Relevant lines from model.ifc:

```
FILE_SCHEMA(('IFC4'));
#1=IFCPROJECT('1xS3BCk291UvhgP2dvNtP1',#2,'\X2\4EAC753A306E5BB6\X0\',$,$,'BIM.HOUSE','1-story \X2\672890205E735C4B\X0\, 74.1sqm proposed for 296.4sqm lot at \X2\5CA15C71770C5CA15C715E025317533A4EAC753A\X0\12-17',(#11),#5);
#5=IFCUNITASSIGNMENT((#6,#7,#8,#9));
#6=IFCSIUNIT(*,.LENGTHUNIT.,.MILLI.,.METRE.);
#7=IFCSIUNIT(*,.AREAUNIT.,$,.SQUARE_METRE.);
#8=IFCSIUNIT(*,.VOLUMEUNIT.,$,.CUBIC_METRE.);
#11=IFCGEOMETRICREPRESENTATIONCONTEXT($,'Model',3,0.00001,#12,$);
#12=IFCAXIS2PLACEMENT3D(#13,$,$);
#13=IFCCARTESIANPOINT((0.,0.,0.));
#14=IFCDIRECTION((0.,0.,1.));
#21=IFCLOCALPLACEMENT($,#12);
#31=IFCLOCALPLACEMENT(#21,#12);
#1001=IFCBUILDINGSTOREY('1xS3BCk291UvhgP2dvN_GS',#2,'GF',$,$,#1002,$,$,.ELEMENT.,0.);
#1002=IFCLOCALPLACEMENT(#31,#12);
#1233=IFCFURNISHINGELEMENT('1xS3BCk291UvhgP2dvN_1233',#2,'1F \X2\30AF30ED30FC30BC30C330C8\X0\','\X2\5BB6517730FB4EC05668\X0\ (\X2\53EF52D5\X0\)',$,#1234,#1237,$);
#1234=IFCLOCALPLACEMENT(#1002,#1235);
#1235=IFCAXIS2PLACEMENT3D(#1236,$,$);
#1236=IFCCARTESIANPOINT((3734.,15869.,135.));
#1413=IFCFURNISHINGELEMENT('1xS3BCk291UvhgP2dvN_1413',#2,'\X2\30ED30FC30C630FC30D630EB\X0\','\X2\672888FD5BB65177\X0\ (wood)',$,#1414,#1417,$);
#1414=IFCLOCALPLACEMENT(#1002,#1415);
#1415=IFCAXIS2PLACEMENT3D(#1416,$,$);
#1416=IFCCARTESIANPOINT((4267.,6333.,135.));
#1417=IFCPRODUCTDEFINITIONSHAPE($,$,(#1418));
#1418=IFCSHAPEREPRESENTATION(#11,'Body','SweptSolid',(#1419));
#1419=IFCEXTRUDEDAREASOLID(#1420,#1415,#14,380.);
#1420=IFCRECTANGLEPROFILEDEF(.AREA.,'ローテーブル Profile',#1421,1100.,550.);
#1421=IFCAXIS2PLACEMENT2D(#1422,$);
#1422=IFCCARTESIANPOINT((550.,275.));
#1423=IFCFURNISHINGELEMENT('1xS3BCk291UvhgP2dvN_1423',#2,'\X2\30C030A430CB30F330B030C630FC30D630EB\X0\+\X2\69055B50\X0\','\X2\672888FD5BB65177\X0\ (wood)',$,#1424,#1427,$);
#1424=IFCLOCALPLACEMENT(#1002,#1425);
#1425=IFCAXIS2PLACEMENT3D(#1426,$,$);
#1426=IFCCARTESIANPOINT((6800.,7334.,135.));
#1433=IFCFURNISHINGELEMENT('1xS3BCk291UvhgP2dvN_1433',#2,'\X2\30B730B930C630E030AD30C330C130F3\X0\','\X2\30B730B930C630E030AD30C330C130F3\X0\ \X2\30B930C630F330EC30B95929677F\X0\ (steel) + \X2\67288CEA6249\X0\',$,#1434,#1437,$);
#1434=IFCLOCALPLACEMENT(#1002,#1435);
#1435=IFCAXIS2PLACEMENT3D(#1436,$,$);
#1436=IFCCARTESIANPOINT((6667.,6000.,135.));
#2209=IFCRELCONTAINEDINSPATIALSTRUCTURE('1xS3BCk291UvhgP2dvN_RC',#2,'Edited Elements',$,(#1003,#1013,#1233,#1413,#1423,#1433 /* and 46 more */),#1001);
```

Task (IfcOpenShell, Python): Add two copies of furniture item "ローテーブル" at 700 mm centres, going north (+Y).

```python
import numpy as np
import ifcopenshell
import ifcopenshell.api.geometry
import ifcopenshell.api.root
import ifcopenshell.util.element
import ifcopenshell.util.placement
import ifcopenshell.util.unit

model = ifcopenshell.open("model.ifc")
unit_scale = ifcopenshell.util.unit.calculate_unit_scale(model)


def reuse_history(source, copy):
    """copy_class also copies each property set's owner history, people and application; keep the originals."""
    for rel in copy.IsDefinedBy:
        if rel.is_a("IfcRelDefinesByProperties") and (history := rel.RelatingPropertyDefinition.OwnerHistory):
            rel.RelatingPropertyDefinition.OwnerHistory = source.OwnerHistory
            ifcopenshell.util.element.remove_deep2(model, history)


source = model.by_guid("1xS3BCk291UvhgP2dvN_1413")
base = ifcopenshell.util.placement.get_local_placement(source.ObjectPlacement)
step = np.array([0.0, 1.0, 0.0]) * 0.7 / unit_scale

for i in range(1, 3):
    copy = ifcopenshell.api.root.copy_class(model, product=source)
    copy.Representation = ifcopenshell.util.element.copy_deep(
        model, source.Representation, exclude=["IfcGeometricRepresentationContext", "IfcRepresentationMap"]
    )
    reuse_history(source, copy)
    matrix = base.copy()
    matrix[:3, 3] += i * step
    print("added at", matrix[:3, 3].round(3) + 0.0)
    ifcopenshell.api.geometry.edit_object_placement(model, product=copy, matrix=matrix, is_si=False)

model.write("model_edited.ifc")
```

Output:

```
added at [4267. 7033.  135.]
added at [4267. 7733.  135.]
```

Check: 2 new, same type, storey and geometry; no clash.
